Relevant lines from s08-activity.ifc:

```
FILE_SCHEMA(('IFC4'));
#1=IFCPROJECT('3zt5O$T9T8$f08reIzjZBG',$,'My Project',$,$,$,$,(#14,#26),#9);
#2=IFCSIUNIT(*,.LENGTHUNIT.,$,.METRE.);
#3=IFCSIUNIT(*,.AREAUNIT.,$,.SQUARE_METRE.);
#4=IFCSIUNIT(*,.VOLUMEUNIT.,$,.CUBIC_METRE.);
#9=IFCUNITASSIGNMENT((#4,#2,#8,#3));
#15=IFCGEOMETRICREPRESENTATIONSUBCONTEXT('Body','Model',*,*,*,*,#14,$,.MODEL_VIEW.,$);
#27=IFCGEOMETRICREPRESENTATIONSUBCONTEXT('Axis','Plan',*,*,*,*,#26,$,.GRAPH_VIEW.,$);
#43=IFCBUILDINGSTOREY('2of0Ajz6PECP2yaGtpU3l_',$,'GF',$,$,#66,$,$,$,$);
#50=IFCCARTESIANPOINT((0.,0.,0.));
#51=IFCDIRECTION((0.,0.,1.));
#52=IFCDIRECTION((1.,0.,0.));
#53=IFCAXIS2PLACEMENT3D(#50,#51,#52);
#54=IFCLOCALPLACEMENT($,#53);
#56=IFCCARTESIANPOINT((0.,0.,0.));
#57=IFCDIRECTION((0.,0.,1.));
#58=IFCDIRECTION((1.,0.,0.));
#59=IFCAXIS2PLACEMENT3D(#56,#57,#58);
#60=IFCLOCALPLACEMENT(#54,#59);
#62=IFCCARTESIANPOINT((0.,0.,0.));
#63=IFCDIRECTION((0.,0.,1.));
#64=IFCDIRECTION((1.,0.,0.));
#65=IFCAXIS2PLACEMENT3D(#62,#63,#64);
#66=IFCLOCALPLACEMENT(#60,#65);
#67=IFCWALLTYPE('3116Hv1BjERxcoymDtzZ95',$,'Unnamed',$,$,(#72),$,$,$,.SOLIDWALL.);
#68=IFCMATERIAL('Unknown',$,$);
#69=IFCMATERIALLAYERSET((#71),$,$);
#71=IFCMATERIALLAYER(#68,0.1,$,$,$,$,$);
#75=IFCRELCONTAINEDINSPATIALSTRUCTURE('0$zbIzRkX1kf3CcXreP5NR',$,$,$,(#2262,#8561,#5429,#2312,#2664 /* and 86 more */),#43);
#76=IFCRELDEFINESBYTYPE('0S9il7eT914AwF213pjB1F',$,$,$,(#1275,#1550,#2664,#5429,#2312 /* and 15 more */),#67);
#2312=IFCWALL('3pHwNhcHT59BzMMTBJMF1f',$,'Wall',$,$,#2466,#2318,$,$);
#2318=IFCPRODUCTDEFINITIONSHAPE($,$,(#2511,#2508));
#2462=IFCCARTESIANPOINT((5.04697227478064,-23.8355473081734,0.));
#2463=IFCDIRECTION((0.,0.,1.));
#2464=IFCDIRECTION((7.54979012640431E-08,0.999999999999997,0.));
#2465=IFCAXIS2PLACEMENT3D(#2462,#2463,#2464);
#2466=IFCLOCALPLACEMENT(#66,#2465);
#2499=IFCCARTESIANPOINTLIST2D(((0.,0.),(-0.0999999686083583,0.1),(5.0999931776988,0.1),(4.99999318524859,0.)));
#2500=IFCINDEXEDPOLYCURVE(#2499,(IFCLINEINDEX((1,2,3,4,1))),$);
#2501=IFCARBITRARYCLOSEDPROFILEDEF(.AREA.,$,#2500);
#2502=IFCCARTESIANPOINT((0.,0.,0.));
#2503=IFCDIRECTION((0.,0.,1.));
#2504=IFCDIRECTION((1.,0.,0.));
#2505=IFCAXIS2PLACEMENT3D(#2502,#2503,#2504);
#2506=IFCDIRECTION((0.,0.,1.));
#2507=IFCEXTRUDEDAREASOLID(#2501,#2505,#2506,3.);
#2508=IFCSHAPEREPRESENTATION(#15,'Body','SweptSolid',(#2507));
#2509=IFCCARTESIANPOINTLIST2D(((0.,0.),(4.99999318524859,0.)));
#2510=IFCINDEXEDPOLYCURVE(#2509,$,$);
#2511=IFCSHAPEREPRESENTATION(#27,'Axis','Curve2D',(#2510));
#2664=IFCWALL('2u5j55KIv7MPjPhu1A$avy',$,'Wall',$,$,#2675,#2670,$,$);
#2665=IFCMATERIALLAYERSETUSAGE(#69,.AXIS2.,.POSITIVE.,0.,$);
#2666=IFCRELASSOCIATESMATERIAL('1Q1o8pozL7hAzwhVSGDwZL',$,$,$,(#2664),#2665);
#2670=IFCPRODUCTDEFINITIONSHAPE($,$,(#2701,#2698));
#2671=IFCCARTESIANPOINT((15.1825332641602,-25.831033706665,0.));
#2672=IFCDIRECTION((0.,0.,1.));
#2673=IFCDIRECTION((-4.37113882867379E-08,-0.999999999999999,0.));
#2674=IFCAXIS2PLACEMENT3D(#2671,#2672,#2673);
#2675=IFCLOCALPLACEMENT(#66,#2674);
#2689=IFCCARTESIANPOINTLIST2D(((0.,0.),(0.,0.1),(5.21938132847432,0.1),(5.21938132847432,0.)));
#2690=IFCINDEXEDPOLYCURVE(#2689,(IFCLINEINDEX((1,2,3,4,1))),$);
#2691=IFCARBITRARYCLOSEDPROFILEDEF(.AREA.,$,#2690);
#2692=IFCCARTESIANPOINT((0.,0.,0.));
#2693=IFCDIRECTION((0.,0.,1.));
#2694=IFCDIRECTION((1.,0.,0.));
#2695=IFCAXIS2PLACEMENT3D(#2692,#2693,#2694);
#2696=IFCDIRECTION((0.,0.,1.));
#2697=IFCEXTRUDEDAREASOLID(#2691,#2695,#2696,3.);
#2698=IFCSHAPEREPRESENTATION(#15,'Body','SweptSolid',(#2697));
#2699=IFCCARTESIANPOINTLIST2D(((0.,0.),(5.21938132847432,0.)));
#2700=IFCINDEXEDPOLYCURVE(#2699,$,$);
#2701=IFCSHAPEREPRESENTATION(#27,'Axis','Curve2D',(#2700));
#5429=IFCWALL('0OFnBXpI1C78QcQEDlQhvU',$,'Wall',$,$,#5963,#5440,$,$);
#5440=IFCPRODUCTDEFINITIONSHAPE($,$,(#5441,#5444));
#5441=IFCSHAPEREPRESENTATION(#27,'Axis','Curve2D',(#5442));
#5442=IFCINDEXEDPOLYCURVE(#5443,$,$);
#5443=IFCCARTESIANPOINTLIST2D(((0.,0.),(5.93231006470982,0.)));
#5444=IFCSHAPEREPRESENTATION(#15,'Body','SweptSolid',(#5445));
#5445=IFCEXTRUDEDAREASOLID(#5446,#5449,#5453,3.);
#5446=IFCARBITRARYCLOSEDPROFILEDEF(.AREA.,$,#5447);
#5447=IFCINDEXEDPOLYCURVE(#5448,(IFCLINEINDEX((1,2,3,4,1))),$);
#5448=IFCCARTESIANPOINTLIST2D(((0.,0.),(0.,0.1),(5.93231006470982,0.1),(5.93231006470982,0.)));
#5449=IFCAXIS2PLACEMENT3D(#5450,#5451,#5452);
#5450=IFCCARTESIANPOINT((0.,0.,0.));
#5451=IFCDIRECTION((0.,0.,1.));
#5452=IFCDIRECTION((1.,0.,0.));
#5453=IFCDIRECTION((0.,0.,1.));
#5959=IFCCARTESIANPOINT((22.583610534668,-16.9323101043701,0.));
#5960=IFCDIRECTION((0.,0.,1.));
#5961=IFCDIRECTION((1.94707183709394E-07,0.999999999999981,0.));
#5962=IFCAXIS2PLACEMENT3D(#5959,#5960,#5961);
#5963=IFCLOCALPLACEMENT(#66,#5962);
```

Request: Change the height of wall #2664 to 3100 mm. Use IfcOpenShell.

```python
import ifcopenshell
import ifcopenshell.geom
import ifcopenshell.util.representation
import ifcopenshell.util.shape
import ifcopenshell.util.unit

model = ifcopenshell.open("s08-activity.ifc")
unit_scale = ifcopenshell.util.unit.calculate_unit_scale(model)
settings = ifcopenshell.geom.settings()


def volume(element):
    """Net volume in cubic metres, openings subtracted."""
    shape = ifcopenshell.geom.create_shape(settings, element)
    return ifcopenshell.util.shape.get_volume(shape.geometry)


wall = model.by_id(2664)
before = volume(wall)

body = ifcopenshell.util.representation.get_representation(wall, "Model", "Body")
solid = body.Items[0]
old_height = solid.Depth
solid.Depth = 3.1 / unit_scale
after = volume(wall)

print(f"height {old_height:g} -> {solid.Depth:g}, volume {before:.3f} -> {after:.3f} m3")

model.write("s08-activity_edited.ifc")
```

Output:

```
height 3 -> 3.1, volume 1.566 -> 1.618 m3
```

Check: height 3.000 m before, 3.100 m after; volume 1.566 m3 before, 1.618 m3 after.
